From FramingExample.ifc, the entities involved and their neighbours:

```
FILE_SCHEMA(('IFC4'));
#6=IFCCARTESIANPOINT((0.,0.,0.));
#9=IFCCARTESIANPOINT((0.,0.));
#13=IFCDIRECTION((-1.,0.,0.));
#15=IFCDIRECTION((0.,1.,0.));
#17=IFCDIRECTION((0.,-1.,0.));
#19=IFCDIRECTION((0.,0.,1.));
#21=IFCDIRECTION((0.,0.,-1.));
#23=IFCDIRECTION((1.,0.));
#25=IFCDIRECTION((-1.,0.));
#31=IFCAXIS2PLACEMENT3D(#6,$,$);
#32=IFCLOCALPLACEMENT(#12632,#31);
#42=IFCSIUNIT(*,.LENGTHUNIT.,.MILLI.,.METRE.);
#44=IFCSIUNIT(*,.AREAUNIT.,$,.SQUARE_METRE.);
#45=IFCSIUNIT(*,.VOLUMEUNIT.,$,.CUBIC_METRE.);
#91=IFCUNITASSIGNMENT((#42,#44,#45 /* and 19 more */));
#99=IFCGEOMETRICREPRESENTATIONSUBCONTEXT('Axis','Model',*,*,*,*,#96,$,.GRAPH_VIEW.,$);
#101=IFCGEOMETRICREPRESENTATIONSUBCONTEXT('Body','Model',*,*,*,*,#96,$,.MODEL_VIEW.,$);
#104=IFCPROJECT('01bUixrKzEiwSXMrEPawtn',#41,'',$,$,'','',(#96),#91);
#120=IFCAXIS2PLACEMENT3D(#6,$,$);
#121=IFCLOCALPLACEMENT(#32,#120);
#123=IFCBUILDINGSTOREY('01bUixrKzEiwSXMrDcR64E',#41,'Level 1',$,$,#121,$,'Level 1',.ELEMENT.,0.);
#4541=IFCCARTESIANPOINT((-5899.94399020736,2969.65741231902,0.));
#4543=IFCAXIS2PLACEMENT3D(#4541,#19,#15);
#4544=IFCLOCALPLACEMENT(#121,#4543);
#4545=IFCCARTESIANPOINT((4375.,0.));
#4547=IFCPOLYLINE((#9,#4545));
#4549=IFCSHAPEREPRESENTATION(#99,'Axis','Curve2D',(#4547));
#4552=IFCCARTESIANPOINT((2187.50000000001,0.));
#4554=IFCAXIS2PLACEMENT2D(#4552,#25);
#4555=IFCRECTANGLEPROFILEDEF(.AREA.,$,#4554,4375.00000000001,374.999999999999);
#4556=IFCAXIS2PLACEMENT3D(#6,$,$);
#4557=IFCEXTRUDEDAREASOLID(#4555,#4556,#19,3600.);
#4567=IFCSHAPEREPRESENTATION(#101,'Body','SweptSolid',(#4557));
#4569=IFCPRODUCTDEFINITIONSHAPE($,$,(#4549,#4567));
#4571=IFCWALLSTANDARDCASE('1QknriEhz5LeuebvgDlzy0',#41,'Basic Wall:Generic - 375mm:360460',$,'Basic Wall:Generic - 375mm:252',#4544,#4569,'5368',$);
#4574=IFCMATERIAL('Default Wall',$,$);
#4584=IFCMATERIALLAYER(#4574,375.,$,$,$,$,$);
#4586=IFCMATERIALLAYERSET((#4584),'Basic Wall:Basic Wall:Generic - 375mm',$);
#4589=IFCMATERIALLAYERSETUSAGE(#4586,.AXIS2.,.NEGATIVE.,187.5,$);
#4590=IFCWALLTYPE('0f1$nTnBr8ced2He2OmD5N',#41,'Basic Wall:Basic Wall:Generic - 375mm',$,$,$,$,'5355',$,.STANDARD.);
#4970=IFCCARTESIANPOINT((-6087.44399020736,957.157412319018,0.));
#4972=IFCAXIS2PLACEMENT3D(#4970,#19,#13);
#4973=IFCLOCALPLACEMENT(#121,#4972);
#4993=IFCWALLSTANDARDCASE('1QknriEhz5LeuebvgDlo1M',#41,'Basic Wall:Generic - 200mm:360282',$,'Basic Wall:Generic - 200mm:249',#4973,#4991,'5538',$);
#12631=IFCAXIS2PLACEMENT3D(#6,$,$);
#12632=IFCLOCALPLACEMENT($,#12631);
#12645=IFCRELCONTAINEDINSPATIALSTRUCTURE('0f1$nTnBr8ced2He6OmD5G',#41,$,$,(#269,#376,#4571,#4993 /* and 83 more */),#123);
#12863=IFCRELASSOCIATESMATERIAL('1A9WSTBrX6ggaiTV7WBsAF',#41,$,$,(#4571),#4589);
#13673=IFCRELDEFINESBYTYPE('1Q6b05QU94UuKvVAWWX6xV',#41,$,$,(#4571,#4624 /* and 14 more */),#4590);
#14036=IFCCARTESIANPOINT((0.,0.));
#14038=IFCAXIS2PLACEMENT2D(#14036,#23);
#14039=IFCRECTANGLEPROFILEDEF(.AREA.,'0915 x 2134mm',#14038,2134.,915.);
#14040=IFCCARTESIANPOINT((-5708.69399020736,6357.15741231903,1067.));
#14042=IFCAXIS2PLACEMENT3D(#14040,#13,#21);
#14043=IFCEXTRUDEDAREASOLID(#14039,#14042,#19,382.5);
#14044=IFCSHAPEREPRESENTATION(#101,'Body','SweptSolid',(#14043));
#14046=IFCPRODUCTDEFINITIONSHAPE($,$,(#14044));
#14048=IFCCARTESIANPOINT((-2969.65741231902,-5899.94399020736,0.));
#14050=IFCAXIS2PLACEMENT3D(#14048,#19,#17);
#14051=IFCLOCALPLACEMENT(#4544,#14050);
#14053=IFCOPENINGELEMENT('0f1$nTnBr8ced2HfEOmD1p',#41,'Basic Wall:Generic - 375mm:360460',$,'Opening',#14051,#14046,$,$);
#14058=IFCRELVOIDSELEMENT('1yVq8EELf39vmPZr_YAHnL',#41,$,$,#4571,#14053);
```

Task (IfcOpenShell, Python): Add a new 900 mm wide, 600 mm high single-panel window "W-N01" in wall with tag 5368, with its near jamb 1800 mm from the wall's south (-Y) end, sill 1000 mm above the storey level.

```python
import numpy as np
import ifcopenshell
import ifcopenshell.api.feature
import ifcopenshell.api.geometry
import ifcopenshell.api.root
import ifcopenshell.api.spatial
import ifcopenshell.geom
import ifcopenshell.util.element
import ifcopenshell.util.placement
import ifcopenshell.util.representation
import ifcopenshell.util.shape
import ifcopenshell.util.unit

model = ifcopenshell.open("FramingExample.ifc")
unit_scale = ifcopenshell.util.unit.calculate_unit_scale(model)
settings = ifcopenshell.geom.settings()


def volume(element):
    """Net volume in cubic metres, openings subtracted."""
    shape = ifcopenshell.geom.create_shape(settings, element)
    return ifcopenshell.util.shape.get_volume(shape.geometry)


wall = model.by_guid("1QknriEhz5LeuebvgDlzy0")
storey = ifcopenshell.util.element.get_container(wall, ifc_class="IfcBuildingStorey")
context = ifcopenshell.util.representation.get_context(model, "Model", "Body", "MODEL_VIEW")
before = volume(wall)

width, height, from_end, sill = 0.9, 0.6, 1.8, 1  # metres

# The wall runs along its own X axis, and the end named is its -X end.
wall_shape = ifcopenshell.geom.create_shape(settings, wall)
x, y, z = ifcopenshell.util.shape.get_vertices(wall_shape.geometry).T
start = x.min() + from_end
face, thickness = float(y.min()), float(y.max() - y.min())
wall_matrix = ifcopenshell.util.placement.get_local_placement(wall.ObjectPlacement)
level = ifcopenshell.util.placement.get_local_placement(storey.ObjectPlacement)[2, 3]


def in_wall(x, y):
    """Placement at x, y metres in the wall's axes, at sill height."""
    matrix = wall_matrix.copy()
    matrix[:, 3] = wall_matrix @ np.array([x / unit_scale, y / unit_scale, 0.0, 1.0])
    matrix[2, 3] = level + sill / unit_scale
    return matrix


# Opening: a box that overshoots both wall faces by 50 mm.
opening = ifcopenshell.api.root.create_entity(model, ifc_class="IfcOpeningElement", predefined_type="OPENING")
box = ifcopenshell.api.geometry.add_wall_representation(
    model, context=context, length=width, height=height, thickness=thickness + 0.1
)
ifcopenshell.api.geometry.assign_representation(model, product=opening, representation=box)
ifcopenshell.api.geometry.edit_object_placement(model, product=opening, matrix=in_wall(start, face - 0.05), is_si=False)
ifcopenshell.api.feature.add_feature(model, feature=opening, element=wall)

window = ifcopenshell.api.root.create_entity(model, ifc_class="IfcWindow", name="W-N01", predefined_type="WINDOW")
window.OverallWidth, window.OverallHeight = width / unit_scale, height / unit_scale
window.PartitioningType = "SINGLE_PANEL"
body = ifcopenshell.api.geometry.add_window_representation(
    model,
    context=context,
    overall_width=window.OverallWidth,
    overall_height=window.OverallHeight,
    partition_type="SINGLE_PANEL",
)
ifcopenshell.api.geometry.assign_representation(model, product=window, representation=body)
ifcopenshell.api.spatial.assign_container(model, products=[window], relating_structure=storey)
ifcopenshell.api.feature.add_filling(model, opening=opening, element=window)

# Centre the window in the wall's thickness.
ifcopenshell.api.geometry.edit_object_placement(model, product=window, matrix=in_wall(start, face), is_si=False)
window_shape = ifcopenshell.geom.create_shape(settings, window)
depth = ifcopenshell.util.shape.get_vertices(window_shape.geometry)[:, 1]
offset = face + thickness / 2 - (depth.min() + depth.max()) / 2
ifcopenshell.api.geometry.edit_object_placement(model, product=window, matrix=in_wall(start, offset), is_si=False)

after = volume(wall)

print(f"wall volume {before:.3f} -> {after:.3f} m3")

model.write("FramingExample_updated.ifc")
```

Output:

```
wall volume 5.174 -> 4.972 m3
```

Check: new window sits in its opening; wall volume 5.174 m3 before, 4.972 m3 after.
